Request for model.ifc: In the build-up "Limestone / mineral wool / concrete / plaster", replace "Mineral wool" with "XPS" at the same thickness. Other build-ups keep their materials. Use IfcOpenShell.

First a look at what the model holds.

```python
import ifcopenshell
import ifcopenshell.util.element

model = ifcopenshell.open("model.ifc")
print(model.schema)
for layer_set in model.by_type("IfcMaterialLayerSet"):
    if layer_set.LayerSetName == "Limestone / mineral wool / concrete / plaster":
        for layer in layer_set.MaterialLayers:
            print(layer.id(), layer.Material and layer.Material.Name, layer.LayerThickness, sep=" | ")
        print(len(ifcopenshell.util.element.get_elements_by_material(model, layer_set)), "elements and types use it")
print(sorted(m.Name for m in model.by_type("IfcMaterial") if m.Name)[:60])
```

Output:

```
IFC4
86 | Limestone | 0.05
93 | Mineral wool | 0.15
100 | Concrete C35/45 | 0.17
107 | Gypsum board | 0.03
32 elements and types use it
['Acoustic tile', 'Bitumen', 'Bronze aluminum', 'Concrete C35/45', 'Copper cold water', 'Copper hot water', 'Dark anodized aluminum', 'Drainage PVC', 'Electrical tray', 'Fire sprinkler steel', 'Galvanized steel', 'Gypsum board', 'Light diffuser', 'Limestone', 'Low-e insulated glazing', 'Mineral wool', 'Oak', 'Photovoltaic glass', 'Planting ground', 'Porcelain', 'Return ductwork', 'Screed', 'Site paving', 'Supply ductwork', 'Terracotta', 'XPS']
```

```python
import ifcopenshell
import ifcopenshell.api.material

model = ifcopenshell.open("model.ifc")

layer_set = next(s for s in model.by_type("IfcMaterialLayerSet") if s.LayerSetName == "Limestone / mineral wool / concrete / plaster")
layer = next(l for l in layer_set.MaterialLayers if l.Material and l.Material.Name == "Mineral wool")
material = next(m for m in model.by_type("IfcMaterial") if m.Name == "XPS")

# Point this one layer at the other material; renaming the old one would change it everywhere.
ifcopenshell.api.material.edit_layer(model, layer=layer, attributes={"Name": material.Name}, material=material)

print([l.Material.Name if l.Material else None for l in layer_set.MaterialLayers])

model.write("model-out.ifc")
```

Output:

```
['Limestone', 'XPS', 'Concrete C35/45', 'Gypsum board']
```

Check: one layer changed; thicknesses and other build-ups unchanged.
